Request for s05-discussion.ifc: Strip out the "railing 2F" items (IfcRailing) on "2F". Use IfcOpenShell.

First a look at what the model holds.

```python
import ifcopenshell
import ifcopenshell.util.element

model = ifcopenshell.open("s05-discussion.ifc")
print(model.schema)
storey = next(s for s in model.by_type("IfcBuildingStorey") if s.Name == "2F")
railings = [e for e in ifcopenshell.util.element.get_decomposition(storey) if e.is_a("IfcRailing")]
seen = {}
for e in railings:
    element_type = ifcopenshell.util.element.get_type(e)
    name = element_type.Name if element_type not in (None, e) else None
    seen[name] = seen.get(name, 0) + 1
for name, count in sorted(seen.items(), key=str):
    print(count, "x", name)
```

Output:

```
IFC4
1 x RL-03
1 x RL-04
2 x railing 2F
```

```python
import ifcopenshell
import ifcopenshell.api.root
import ifcopenshell.util.element

model = ifcopenshell.open("s05-discussion.ifc")

storey = next(s for s in model.by_type("IfcBuildingStorey") if s.Name == "2F")
railings = [e for e in ifcopenshell.util.element.get_decomposition(storey) if e.is_a("IfcRailing")]
targets = [e for e in railings if (t := ifcopenshell.util.element.get_type(e)) not in (None, e) and t.Name == "railing 2F"]

for e in targets:
    ifcopenshell.api.root.remove_product(model, product=e)
print(len(targets), "removed")

model.write("s05-discussion_v2.ifc")
```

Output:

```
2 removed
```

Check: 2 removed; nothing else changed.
